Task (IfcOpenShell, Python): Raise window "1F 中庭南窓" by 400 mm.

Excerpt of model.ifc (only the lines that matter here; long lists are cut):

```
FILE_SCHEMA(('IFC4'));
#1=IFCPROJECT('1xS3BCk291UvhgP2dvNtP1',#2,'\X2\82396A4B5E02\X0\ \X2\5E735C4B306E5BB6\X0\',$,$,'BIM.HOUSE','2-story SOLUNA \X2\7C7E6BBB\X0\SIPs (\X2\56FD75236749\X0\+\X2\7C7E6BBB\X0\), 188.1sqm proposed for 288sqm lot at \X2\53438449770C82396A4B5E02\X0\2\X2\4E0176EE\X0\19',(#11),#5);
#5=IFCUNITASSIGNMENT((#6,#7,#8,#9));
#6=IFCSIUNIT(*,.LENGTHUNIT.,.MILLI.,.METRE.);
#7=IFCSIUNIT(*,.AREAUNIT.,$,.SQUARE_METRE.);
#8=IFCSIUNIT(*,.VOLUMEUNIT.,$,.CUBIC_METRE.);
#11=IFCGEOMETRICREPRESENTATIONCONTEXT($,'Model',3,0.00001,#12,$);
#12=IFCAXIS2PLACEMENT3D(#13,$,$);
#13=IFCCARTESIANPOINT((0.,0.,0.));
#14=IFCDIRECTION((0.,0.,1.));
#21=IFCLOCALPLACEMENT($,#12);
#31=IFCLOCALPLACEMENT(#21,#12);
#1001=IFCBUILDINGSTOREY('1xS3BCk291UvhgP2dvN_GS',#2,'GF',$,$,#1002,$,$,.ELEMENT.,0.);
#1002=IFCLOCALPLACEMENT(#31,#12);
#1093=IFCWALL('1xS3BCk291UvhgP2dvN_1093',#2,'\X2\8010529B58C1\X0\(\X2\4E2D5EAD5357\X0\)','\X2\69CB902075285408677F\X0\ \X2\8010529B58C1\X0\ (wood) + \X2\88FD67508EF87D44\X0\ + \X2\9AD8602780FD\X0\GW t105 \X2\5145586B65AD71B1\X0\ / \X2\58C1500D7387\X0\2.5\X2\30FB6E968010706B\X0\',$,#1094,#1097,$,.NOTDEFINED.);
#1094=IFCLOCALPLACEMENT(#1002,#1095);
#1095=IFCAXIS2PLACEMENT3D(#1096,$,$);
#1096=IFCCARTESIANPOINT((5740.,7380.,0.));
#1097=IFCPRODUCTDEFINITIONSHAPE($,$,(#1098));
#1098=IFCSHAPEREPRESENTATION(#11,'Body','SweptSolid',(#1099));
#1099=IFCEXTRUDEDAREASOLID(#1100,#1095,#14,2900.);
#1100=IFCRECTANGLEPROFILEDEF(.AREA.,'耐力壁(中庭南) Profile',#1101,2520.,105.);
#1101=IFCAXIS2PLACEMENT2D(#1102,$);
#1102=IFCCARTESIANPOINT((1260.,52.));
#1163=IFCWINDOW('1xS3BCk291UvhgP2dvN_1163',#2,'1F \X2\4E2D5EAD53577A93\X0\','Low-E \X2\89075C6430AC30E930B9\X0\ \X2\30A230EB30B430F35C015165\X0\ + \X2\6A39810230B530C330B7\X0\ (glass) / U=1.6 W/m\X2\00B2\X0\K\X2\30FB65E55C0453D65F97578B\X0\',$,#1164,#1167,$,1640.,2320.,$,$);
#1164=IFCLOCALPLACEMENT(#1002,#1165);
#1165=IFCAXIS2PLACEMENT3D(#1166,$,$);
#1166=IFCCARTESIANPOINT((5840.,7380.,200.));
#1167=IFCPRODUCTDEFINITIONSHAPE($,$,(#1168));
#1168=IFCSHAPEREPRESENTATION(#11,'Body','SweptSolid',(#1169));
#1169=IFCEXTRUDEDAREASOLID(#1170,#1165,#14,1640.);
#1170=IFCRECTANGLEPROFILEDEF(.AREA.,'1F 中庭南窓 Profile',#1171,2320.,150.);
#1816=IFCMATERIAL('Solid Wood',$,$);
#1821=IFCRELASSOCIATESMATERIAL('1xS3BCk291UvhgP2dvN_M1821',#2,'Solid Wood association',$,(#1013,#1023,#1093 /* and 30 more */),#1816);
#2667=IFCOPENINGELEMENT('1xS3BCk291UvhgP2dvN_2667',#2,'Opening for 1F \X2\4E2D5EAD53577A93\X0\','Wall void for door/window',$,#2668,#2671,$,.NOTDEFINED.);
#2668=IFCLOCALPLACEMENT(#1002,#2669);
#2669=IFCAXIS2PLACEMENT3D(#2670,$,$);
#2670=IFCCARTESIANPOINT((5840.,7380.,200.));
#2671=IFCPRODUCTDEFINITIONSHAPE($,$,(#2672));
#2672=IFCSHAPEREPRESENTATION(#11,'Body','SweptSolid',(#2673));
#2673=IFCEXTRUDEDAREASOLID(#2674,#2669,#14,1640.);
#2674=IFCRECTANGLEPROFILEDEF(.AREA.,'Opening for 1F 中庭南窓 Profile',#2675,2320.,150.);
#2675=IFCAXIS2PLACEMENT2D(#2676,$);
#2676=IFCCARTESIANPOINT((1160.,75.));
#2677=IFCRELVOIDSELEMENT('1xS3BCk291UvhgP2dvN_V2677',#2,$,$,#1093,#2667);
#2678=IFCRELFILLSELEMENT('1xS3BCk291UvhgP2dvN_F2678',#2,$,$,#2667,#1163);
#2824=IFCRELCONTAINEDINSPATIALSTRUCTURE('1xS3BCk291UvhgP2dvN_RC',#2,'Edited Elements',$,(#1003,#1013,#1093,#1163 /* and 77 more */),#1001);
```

```python
import numpy as np
import ifcopenshell
import ifcopenshell.api.geometry
import ifcopenshell.util.placement
import ifcopenshell.util.unit

model = ifcopenshell.open("model.ifc")
unit_scale = ifcopenshell.util.unit.calculate_unit_scale(model)

window = model.by_id(1163)
opening = window.FillsVoids[0].RelatingOpeningElement
dz = 0.4 / unit_scale

shift = np.array([0.0, 0.0, dz])
# The window is not placed relative to its opening, so move both.
for product in (opening, window):
    matrix = ifcopenshell.util.placement.get_local_placement(product.ObjectPlacement)
    matrix[:3, 3] += shift
    ifcopenshell.api.geometry.edit_object_placement(model, product=product, matrix=matrix, is_si=False)

print(f"moved by {dz * unit_scale:+.3f} m")

model.write("model-out.ifc")
```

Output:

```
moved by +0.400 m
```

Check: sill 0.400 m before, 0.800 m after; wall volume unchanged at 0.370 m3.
